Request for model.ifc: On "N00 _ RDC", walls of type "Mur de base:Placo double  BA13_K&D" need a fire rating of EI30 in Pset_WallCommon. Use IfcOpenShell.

First a look at what the model holds.

```python
import ifcopenshell
import ifcopenshell.util.element

model = ifcopenshell.open("model.ifc")
print(model.schema)
storey = next(s for s in model.by_type("IfcBuildingStorey") if s.Name == "N00 _ RDC")
walls = [e for e in ifcopenshell.util.element.get_decomposition(storey) if e.is_a("IfcWall")]
seen = {}
for e in walls:
    element_type = ifcopenshell.util.element.get_type(e)
    key = (element_type.Name if element_type != e and element_type else None, ifcopenshell.util.element.get_pset(e, "Pset_WallCommon", "FireRating"))
    seen[key] = seen.get(key, 0) + 1
for (name, value), count in sorted(seen.items(), key=str):
    print(count, "x", name, "|", value)
```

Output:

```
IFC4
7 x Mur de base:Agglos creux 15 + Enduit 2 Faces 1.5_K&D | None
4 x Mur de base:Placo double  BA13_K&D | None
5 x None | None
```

```python
import ifcopenshell
import ifcopenshell.api.pset
import ifcopenshell.util.element

model = ifcopenshell.open("model.ifc")

storey = next(s for s in model.by_type("IfcBuildingStorey") if s.Name == "N00 _ RDC")
walls = [e for e in ifcopenshell.util.element.get_decomposition(storey) if e.is_a("IfcWall")]

count = 0
for e in walls:
    element_type = ifcopenshell.util.element.get_type(e)
    if element_type in (None, e) or element_type.Name != "Mur de base:Placo double  BA13_K&D":
        continue
    # add_pset returns the element's existing set when there is one.
    pset = ifcopenshell.api.pset.add_pset(model, product=e, name="Pset_WallCommon")
    ifcopenshell.api.pset.edit_pset(model, pset=pset, properties={"FireRating": "EI30"})
    count += 1

print(count, "walls updated")

model.write("model_updated.ifc")
```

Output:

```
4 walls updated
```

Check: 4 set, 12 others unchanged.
